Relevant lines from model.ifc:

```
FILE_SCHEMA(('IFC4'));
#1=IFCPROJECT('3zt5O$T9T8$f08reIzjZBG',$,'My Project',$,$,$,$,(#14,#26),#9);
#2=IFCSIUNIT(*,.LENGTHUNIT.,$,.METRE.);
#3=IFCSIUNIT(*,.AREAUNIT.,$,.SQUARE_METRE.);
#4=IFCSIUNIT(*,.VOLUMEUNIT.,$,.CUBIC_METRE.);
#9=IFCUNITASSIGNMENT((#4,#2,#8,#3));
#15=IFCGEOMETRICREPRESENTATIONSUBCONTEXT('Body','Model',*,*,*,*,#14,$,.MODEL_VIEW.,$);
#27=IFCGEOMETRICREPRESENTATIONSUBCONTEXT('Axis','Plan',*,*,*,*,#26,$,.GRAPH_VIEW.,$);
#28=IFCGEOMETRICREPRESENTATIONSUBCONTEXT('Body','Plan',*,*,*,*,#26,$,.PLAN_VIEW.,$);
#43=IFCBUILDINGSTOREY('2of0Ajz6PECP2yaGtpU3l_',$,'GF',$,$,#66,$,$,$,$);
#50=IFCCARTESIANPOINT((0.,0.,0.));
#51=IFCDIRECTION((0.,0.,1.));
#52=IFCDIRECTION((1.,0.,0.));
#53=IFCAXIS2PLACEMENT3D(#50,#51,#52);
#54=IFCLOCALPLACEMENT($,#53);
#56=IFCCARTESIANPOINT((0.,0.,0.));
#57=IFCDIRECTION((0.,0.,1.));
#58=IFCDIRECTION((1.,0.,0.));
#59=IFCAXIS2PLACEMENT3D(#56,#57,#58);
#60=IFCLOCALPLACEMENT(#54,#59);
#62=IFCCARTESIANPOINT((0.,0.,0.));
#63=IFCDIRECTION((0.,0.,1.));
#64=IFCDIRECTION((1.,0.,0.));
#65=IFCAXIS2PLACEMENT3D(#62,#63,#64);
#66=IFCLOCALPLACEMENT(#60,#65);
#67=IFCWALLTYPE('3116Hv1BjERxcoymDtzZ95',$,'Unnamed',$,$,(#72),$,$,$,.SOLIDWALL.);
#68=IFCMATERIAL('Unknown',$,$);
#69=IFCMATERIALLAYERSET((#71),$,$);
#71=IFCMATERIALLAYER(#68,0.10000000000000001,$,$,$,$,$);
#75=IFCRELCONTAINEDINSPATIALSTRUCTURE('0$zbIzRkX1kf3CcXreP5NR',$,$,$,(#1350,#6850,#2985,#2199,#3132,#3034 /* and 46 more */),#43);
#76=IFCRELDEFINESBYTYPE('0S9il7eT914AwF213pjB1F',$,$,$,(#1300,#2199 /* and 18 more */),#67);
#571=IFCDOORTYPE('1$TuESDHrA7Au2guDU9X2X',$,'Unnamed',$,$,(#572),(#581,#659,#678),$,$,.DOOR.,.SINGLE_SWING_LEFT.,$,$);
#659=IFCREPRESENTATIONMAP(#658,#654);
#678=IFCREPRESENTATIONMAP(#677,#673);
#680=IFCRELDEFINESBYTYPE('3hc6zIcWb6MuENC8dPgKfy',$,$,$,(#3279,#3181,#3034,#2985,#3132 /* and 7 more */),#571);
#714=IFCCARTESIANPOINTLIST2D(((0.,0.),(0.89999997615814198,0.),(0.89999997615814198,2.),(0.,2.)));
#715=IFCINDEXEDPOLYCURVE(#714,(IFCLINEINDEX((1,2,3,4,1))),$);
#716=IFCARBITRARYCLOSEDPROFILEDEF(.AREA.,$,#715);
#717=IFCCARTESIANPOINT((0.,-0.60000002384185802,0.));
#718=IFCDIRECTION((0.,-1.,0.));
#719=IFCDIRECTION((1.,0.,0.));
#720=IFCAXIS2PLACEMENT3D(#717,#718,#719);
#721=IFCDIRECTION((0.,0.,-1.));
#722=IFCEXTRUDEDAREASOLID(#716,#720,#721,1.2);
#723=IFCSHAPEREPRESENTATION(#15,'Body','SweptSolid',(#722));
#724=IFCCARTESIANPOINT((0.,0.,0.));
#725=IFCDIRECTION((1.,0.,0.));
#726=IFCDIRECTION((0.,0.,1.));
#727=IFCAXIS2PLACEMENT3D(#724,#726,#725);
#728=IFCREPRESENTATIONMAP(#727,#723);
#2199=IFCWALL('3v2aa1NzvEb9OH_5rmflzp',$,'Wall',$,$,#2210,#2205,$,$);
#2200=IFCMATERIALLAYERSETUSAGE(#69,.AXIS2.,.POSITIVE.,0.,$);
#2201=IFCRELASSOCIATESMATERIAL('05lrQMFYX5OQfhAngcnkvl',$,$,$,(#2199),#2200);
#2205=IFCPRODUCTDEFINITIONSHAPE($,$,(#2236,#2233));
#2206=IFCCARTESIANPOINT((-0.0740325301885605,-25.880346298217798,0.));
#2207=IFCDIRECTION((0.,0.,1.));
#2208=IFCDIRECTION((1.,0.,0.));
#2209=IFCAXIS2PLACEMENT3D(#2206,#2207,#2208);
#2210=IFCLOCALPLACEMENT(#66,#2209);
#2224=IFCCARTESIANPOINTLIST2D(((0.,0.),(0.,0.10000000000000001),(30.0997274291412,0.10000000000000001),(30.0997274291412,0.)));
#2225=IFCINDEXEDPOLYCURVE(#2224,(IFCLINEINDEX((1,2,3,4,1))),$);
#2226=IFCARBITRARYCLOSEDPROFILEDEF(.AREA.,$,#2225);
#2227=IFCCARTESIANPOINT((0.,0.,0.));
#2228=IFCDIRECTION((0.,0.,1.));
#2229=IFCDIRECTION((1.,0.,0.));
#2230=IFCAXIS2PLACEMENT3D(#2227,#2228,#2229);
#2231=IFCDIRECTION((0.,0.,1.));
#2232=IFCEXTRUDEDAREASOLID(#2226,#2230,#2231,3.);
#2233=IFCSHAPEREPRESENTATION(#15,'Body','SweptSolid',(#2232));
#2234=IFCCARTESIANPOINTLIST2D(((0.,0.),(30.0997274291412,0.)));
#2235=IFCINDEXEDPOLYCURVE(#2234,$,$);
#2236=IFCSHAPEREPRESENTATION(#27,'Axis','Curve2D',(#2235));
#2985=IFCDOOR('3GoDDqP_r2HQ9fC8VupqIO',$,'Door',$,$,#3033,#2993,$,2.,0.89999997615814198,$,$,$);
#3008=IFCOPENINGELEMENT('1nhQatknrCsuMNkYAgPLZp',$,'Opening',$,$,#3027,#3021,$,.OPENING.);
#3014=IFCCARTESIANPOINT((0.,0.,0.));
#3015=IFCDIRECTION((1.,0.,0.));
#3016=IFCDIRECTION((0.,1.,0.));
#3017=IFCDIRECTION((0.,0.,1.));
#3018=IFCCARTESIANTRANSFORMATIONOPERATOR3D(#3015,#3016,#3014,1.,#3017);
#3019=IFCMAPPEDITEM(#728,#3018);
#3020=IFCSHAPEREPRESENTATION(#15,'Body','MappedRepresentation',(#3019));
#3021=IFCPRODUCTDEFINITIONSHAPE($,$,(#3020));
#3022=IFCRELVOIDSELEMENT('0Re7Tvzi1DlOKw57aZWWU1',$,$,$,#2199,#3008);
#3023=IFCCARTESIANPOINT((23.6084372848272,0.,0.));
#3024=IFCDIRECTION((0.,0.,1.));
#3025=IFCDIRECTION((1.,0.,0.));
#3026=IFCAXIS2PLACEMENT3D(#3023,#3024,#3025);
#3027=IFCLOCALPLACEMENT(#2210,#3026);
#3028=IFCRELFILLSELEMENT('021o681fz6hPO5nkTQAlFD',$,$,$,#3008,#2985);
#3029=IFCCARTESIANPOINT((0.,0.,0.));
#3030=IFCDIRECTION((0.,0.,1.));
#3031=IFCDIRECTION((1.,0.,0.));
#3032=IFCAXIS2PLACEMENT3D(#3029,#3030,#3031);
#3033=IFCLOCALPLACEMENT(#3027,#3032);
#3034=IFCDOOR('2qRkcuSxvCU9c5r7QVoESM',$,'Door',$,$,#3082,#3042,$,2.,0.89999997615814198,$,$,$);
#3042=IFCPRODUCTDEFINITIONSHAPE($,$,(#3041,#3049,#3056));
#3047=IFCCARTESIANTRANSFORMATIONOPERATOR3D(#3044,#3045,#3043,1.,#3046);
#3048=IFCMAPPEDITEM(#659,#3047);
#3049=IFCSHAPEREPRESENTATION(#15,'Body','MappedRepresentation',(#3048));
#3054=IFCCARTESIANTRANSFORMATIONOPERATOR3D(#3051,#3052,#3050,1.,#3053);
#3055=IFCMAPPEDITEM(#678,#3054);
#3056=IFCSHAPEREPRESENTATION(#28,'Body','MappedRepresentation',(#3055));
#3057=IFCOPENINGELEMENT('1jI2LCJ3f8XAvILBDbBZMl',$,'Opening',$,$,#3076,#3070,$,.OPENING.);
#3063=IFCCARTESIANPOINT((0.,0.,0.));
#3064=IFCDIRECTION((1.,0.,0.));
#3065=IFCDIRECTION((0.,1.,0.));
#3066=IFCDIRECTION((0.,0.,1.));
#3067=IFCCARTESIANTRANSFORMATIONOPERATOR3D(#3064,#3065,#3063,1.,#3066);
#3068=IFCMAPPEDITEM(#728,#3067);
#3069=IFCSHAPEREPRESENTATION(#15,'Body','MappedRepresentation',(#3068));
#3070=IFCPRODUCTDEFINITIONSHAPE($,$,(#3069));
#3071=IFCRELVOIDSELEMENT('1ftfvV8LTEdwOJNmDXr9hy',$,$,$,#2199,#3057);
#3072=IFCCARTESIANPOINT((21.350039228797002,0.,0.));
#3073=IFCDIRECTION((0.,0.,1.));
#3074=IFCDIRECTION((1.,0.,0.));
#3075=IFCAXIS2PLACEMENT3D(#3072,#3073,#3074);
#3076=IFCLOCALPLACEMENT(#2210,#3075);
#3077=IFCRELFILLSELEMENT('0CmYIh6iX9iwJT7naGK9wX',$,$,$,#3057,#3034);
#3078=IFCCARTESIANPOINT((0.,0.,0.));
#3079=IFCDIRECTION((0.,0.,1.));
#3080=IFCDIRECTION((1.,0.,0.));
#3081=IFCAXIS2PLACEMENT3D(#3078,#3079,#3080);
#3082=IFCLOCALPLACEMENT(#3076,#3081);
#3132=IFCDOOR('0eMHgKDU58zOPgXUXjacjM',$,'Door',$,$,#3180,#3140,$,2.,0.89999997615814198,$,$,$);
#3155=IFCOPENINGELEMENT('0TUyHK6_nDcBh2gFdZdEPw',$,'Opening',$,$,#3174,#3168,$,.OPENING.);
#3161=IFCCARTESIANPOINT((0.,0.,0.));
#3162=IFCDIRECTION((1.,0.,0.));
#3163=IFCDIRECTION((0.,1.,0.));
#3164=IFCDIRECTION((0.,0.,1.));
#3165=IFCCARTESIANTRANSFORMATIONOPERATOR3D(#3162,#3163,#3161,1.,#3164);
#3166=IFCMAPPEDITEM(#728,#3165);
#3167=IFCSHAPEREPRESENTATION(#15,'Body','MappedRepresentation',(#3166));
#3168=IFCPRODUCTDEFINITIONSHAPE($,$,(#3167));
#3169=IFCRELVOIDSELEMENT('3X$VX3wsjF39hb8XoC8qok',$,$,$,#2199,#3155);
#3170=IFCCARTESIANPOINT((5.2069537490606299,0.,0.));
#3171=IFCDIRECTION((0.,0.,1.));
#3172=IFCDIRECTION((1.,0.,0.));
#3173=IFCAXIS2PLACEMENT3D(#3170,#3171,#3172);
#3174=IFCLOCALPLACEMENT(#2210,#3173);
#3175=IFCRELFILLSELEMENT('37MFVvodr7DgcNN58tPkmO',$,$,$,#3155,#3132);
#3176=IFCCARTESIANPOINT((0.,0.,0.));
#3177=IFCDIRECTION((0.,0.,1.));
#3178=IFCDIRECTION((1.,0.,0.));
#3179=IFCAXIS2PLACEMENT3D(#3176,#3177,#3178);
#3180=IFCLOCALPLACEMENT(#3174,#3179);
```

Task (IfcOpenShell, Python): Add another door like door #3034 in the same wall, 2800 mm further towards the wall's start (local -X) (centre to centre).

```python
import ifcopenshell
import ifcopenshell.api.feature
import ifcopenshell.api.geometry
import ifcopenshell.api.root
import ifcopenshell.geom
import ifcopenshell.util.element
import ifcopenshell.util.placement
import ifcopenshell.util.shape

model = ifcopenshell.open("model.ifc")
settings = ifcopenshell.geom.settings()


def volume(element):
    """Net volume in cubic metres, openings subtracted."""
    shape = ifcopenshell.geom.create_shape(settings, element)
    return ifcopenshell.util.shape.get_volume(shape.geometry)


door = model.by_guid("2qRkcuSxvCU9c5r7QVoESM")
opening = door.FillsVoids[0].RelatingOpeningElement
wall = opening.VoidsElements[0].RelatingBuildingElement
before = volume(wall)
shift = ifcopenshell.util.placement.get_local_placement(wall.ObjectPlacement)[:3, 0] * -2.8

# copy_class copies the void relationship, type, container and properties, but no geometry.
new_opening = ifcopenshell.api.root.copy_class(model, product=opening)
new_opening.Representation = ifcopenshell.util.element.copy_deep(
    model, opening.Representation, exclude=["IfcGeometricRepresentationContext", "IfcRepresentationMap"]
)
new_door = ifcopenshell.api.root.copy_class(model, product=door)
new_door.Representation = ifcopenshell.util.element.copy_deep(
    model, door.Representation, exclude=["IfcGeometricRepresentationContext", "IfcRepresentationMap"]
)
ifcopenshell.api.feature.add_filling(model, opening=new_opening, element=new_door)

for old, new in ((opening, new_opening), (door, new_door)):
    matrix = ifcopenshell.util.placement.get_local_placement(old.ObjectPlacement)
    matrix[:3, 3] += shift
    ifcopenshell.api.geometry.edit_object_placement(model, product=new, matrix=matrix, is_si=False)

after = volume(wall)

print(f"wall volume {before:.3f} -> {after:.3f} m3")

model.write("model-out.ifc")
```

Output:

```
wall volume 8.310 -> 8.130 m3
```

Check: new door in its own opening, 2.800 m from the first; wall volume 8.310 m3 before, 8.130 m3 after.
